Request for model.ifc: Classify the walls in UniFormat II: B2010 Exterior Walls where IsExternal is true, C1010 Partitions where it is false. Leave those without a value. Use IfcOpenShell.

First a look at what the model holds.

```python
import ifcopenshell
import ifcopenshell.util.element

model = ifcopenshell.open("model.ifc")
print(model.schema)
print("classifications:", [c.Name for c in model.by_type("IfcClassification")])
values = [ifcopenshell.util.element.get_pset(e, "Pset_WallCommon", "IsExternal") for e in model.by_type("IfcWall")]
for value in (True, False, None):
    print("IsExternal", value, values.count(value))
```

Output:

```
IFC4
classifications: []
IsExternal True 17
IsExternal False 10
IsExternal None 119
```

```python
import ifcopenshell
import ifcopenshell.api.classification
import ifcopenshell.util.element

model = ifcopenshell.open("model.ifc")

system = ifcopenshell.api.classification.add_classification(model, classification="UniFormat II")

walls = model.by_type("IfcWall")
external = {e: ifcopenshell.util.element.get_pset(e, "Pset_WallCommon", "IsExternal") for e in walls}
for flag, code, name in ((True, "B2010", "Exterior Walls"), (False, "C1010", "Partitions")):
    products = [e for e in walls if external[e] is flag]
    ifcopenshell.api.classification.add_reference(
        model, products=products, classification=system, identification=code, name=name
    )
    print(code, len(products))

model.write("model_updated.ifc")
```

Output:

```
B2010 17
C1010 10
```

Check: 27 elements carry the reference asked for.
